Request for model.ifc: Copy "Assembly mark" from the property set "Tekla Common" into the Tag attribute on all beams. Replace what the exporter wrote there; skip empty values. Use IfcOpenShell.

First a look at what the model holds.

```python
import ifcopenshell
import ifcopenshell.util.element

model = ifcopenshell.open("model.ifc")
print(model.schema)
beams = model.by_type("IfcBeam")
print(len(beams), "beams")
for e in beams[:8]:
    source = ifcopenshell.util.element.get_pset(e, "Tekla Common", "Assembly mark")
    target = e.Tag
    print(e.id(), repr(source), repr(target), sep=" | ")
```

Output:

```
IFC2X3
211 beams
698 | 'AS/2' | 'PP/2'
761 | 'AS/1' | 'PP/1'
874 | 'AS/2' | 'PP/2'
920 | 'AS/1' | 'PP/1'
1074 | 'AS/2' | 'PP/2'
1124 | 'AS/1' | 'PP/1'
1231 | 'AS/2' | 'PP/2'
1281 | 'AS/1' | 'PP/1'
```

```python
import ifcopenshell
import ifcopenshell.util.element

model = ifcopenshell.open("model.ifc")

count = 0
for e in model.by_type("IfcBeam"):
    value = ifcopenshell.util.element.get_pset(e, "Tekla Common", "Assembly mark")
    current = e.Tag
    if not value or not value.strip() or current == value:
        continue
    e.Tag = value
    count += 1

print(count, "beams updated")

model.write("model_v2.ifc")
```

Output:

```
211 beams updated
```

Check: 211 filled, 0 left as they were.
